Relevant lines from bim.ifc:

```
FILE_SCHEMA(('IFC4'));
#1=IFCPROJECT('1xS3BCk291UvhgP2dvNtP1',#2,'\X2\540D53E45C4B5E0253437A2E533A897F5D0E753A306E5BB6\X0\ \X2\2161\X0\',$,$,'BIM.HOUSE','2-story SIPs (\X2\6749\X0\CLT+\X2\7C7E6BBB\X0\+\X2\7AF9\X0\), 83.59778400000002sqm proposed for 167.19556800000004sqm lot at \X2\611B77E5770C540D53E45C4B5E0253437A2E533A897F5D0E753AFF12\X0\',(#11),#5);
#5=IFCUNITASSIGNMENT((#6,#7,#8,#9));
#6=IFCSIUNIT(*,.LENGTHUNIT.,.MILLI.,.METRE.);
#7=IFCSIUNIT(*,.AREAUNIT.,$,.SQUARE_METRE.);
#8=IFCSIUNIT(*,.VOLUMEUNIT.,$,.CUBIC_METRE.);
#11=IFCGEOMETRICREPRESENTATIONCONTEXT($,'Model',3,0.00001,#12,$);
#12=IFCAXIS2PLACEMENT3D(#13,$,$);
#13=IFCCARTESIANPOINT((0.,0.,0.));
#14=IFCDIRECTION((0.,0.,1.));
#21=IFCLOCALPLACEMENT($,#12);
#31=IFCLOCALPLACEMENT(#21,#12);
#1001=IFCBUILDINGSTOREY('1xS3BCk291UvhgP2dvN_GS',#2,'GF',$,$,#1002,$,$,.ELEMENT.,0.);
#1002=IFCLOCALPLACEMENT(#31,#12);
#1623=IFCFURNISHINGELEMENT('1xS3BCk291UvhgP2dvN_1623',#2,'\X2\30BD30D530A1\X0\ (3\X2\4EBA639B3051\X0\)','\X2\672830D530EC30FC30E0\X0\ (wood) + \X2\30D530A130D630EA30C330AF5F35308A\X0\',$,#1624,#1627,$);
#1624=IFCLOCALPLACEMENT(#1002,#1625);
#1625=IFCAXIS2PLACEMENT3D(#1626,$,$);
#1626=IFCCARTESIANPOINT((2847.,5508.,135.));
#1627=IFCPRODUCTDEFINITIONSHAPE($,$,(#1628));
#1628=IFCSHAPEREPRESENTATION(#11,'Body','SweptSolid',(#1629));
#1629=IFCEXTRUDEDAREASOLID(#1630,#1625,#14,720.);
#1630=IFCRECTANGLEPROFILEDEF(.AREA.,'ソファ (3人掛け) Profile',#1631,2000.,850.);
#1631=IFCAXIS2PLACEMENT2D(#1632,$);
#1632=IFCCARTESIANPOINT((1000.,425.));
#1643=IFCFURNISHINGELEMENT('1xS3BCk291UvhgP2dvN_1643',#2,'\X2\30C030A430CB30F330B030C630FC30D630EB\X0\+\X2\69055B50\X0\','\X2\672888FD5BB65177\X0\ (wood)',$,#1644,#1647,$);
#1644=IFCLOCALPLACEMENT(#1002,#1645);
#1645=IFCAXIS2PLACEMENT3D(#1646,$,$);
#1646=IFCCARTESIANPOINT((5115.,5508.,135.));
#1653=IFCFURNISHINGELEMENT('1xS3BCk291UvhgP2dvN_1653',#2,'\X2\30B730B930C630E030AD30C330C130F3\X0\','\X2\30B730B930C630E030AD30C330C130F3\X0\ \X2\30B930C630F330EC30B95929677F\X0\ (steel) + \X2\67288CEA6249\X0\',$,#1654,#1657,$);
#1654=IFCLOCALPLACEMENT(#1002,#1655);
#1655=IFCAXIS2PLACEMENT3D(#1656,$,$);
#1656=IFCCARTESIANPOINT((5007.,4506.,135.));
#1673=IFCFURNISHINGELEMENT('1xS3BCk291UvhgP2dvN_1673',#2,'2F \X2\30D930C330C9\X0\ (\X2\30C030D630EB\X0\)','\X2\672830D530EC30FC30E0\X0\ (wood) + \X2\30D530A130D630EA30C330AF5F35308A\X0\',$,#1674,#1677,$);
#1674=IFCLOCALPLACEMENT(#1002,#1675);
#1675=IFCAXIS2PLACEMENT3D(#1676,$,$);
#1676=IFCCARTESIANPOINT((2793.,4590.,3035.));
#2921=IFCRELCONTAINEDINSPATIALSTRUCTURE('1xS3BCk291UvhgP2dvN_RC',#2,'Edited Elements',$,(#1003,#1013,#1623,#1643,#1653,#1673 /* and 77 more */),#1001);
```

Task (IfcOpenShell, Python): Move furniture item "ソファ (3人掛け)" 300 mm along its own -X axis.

```python
import ifcopenshell
import ifcopenshell.api.geometry
import ifcopenshell.util.placement

model = ifcopenshell.open("bim.ifc")

item = model.by_guid("1xS3BCk291UvhgP2dvN_1623")
matrix = ifcopenshell.util.placement.get_local_placement(item.ObjectPlacement)
matrix[:3, 3] -= matrix[:3, 0] * 300.0
ifcopenshell.api.geometry.edit_object_placement(model, product=item, matrix=matrix, is_si=False)

print(ifcopenshell.util.placement.get_local_placement(item.ObjectPlacement).round(3) + 0.0)

model.write("bim_edited.ifc")
```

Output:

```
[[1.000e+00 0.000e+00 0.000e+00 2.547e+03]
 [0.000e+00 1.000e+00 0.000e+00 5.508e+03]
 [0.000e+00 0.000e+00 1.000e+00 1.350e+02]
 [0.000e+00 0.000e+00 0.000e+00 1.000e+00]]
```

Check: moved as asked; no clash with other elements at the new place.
